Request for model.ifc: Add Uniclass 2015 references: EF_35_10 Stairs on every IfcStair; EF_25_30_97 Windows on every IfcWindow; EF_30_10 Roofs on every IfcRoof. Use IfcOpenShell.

First a look at what the model holds.

```python
import ifcopenshell

model = ifcopenshell.open("model.ifc")
print(model.schema)
print("classifications:", [c.Name for c in model.by_type("IfcClassification")])
for ifc_class in ("IfcDoor", "IfcRoof", "IfcStair", "IfcWall", "IfcWindow"):
    print(ifc_class, len(model.by_type(ifc_class)))
```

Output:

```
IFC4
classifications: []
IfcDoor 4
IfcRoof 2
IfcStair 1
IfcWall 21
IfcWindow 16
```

```python
import ifcopenshell
import ifcopenshell.api.classification

model = ifcopenshell.open("model.ifc")

system = ifcopenshell.api.classification.add_classification(model, classification="Uniclass 2015")

codes = {
    "IfcStair": ("EF_35_10", "Stairs"),
    "IfcWindow": ("EF_25_30_97", "Windows"),
    "IfcRoof": ("EF_30_10", "Roofs"),
}
for ifc_class, (code, name) in codes.items():
    products = model.by_type(ifc_class)
    ifcopenshell.api.classification.add_reference(
        model, products=products, classification=system, identification=code, name=name
    )
    print(code, len(products))

model.write("model_rev.ifc")
```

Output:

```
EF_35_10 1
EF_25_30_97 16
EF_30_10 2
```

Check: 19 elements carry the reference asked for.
